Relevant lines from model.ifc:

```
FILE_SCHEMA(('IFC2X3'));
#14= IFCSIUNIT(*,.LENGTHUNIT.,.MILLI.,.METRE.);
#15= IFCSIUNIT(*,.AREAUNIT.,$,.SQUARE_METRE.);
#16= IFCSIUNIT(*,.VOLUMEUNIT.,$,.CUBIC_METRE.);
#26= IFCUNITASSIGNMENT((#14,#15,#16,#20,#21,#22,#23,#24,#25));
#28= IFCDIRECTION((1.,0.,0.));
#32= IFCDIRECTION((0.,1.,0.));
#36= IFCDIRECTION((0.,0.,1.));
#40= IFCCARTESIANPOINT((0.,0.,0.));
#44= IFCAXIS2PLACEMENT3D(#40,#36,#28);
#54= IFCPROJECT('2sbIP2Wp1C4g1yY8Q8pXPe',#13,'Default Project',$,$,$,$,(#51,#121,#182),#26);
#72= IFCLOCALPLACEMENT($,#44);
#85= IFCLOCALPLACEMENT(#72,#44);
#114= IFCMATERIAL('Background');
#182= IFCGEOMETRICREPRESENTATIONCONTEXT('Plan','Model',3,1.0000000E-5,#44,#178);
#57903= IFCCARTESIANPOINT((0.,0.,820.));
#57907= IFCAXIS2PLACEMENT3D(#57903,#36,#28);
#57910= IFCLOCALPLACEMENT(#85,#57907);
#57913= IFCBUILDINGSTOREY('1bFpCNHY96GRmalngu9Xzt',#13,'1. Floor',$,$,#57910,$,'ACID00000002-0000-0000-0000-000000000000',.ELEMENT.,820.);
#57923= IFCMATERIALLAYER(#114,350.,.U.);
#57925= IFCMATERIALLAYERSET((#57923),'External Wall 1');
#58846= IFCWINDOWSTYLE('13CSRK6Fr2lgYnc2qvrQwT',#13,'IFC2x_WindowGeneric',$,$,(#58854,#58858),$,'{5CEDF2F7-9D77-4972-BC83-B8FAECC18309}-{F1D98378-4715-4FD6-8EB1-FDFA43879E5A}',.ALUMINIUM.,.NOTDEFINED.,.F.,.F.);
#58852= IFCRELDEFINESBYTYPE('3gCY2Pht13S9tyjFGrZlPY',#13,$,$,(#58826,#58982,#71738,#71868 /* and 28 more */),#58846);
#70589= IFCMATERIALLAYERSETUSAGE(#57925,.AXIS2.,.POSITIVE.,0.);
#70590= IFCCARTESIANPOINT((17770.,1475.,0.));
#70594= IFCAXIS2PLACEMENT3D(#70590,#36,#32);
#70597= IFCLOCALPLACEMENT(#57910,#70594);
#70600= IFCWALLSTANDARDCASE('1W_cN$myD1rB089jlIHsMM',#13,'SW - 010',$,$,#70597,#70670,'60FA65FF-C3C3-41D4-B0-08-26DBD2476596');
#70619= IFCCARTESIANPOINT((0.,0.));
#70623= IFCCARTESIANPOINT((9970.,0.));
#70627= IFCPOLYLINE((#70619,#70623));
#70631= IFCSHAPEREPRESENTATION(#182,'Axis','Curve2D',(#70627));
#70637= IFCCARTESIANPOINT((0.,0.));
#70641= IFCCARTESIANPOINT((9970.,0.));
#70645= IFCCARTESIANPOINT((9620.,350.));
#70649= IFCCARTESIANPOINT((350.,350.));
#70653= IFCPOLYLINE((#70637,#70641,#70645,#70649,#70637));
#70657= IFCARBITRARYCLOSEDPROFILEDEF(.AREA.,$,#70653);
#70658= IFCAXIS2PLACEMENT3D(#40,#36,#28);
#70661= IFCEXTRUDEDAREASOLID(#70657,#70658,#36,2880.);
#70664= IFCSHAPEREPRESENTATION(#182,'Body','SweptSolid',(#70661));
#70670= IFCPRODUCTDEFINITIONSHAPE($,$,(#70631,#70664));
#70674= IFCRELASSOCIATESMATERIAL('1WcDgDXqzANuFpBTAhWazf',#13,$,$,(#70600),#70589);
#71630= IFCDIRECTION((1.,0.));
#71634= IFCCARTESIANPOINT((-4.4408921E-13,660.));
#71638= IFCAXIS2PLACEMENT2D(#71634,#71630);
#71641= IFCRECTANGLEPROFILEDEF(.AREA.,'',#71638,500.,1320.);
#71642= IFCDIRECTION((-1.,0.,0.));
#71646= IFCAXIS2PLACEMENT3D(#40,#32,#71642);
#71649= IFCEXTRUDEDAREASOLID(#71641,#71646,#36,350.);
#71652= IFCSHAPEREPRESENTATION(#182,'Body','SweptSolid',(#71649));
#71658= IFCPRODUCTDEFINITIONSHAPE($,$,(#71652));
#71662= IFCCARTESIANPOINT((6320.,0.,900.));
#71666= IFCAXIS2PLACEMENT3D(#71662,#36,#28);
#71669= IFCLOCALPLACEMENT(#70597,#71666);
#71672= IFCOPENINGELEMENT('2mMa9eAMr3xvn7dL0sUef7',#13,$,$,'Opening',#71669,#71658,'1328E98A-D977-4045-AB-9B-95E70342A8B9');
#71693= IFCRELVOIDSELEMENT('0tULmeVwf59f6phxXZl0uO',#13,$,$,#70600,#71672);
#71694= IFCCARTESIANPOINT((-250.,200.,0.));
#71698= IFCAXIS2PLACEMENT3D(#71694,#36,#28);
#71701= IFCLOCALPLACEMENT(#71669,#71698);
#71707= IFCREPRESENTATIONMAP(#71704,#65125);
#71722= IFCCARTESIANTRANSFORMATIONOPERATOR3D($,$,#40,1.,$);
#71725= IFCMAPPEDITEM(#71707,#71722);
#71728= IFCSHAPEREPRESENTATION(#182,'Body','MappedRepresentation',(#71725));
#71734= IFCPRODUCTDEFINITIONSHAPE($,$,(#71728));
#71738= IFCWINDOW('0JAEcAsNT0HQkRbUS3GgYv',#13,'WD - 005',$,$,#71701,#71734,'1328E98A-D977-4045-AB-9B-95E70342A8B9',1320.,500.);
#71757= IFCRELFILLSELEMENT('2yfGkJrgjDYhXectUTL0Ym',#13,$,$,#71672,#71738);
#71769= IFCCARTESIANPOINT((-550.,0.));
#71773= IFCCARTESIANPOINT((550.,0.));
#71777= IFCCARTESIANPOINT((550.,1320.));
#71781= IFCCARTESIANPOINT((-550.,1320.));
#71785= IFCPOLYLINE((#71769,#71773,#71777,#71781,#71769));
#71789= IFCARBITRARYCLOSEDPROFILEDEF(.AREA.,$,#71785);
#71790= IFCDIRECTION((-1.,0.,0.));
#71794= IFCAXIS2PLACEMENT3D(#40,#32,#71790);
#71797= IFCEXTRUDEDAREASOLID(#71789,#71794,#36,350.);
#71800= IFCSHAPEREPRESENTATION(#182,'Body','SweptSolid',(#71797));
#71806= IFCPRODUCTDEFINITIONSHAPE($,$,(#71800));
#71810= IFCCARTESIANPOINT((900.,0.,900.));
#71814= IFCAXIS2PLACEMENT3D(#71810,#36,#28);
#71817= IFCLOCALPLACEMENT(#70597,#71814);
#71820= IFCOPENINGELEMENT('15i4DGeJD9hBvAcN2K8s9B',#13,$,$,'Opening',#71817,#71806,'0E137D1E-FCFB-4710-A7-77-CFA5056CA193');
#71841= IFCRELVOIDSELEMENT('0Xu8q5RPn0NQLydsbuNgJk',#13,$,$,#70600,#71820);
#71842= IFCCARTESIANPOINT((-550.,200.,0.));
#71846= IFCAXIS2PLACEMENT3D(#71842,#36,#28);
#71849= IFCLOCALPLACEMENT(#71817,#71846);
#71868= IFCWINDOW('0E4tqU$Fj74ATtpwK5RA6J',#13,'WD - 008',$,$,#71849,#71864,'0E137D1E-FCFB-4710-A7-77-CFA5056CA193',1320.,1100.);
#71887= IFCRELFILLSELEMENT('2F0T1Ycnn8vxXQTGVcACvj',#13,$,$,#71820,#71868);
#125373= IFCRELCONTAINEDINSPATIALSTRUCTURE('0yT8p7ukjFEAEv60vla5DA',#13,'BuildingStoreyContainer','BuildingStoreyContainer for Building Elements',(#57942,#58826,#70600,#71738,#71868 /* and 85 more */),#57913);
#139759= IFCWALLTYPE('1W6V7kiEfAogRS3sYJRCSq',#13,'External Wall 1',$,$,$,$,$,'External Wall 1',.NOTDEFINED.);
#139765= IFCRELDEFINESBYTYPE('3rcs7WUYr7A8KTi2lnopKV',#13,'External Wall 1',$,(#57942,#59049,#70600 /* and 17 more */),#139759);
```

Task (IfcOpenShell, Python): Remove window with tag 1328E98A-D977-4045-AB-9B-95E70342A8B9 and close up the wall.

```python
import ifcopenshell
import ifcopenshell.api.feature
import ifcopenshell.api.root
import ifcopenshell.geom
import ifcopenshell.util.shape

model = ifcopenshell.open("model.ifc")
settings = ifcopenshell.geom.settings()


def volume(element):
    """Net volume in cubic metres, openings subtracted."""
    shape = ifcopenshell.geom.create_shape(settings, element)
    return ifcopenshell.util.shape.get_volume(shape.geometry)


window = model.by_guid("0JAEcAsNT0HQkRbUS3GgYv")
opening = window.FillsVoids[0].RelatingOpeningElement
wall = opening.VoidsElements[0].RelatingBuildingElement
before = volume(wall)

ifcopenshell.api.root.remove_product(model, product=window)
ifcopenshell.api.feature.remove_feature(model, feature=opening)

after = volume(wall)

print(f"wall volume {before:.3f} -> {after:.3f} m3")

model.write("model-out.ifc")
```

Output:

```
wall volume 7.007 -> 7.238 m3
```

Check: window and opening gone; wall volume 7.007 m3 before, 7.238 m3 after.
